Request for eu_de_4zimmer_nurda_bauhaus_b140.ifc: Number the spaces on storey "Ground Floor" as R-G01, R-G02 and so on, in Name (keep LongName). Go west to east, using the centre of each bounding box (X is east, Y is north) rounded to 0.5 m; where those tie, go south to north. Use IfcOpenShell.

First a look at what the model holds.

```python
import ifcopenshell
import ifcopenshell.util.element
import ifcopenshell.util.placement

model = ifcopenshell.open("eu_de_4zimmer_nurda_bauhaus_b140.ifc")
print(model.schema)
storey = next(s for s in model.by_type("IfcBuildingStorey") if s.Name == "Ground Floor")
spaces = [e for e in ifcopenshell.util.element.get_decomposition(storey) if e.is_a("IfcSpace")]
for e in sorted(spaces, key=lambda e: e.id()):
    origin = ifcopenshell.util.placement.get_local_placement(e.ObjectPlacement)[:3, 3]
    print(e.id(), e.Name, e.LongName, origin.round(2) + 0.0, sep=" | ")
```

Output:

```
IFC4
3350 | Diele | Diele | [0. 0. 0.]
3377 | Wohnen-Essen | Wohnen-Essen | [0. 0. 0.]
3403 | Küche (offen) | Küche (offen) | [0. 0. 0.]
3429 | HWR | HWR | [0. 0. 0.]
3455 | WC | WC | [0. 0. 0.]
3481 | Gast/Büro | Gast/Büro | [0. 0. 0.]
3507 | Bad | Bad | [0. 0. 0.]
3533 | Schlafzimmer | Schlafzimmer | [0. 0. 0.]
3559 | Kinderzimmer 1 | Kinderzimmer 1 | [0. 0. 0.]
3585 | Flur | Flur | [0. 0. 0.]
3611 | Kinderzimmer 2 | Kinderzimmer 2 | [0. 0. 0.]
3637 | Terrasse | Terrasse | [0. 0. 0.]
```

```python
import ifcopenshell
import ifcopenshell.geom
import ifcopenshell.util.element
import ifcopenshell.util.shape

model = ifcopenshell.open("eu_de_4zimmer_nurda_bauhaus_b140.ifc")
settings = ifcopenshell.geom.settings()
settings.set("use-world-coords", True)


def centre(element):
    shape = ifcopenshell.geom.create_shape(settings, element)
    return ifcopenshell.util.shape.get_bbox_centroid(shape.geometry)


storey = next(s for s in model.by_type("IfcBuildingStorey") if s.Name == "Ground Floor")
spaces = [e for e in ifcopenshell.util.element.get_decomposition(storey) if e.is_a("IfcSpace")]

# Insertion points can sit at a corner or the storey origin, so sort by the geometry (in metres).
centres = {e: centre(e) for e in spaces}
spaces.sort(key=lambda e: (round(centres[e][0] / 0.5), centres[e][1]))

for i, e in enumerate(spaces, start=1):
    number = f"R-G{i:02d}"
    e.Name = number
    print(e.id(), number)

model.write("eu_de_4zimmer_nurda_bauhaus_b140-out.ifc")
```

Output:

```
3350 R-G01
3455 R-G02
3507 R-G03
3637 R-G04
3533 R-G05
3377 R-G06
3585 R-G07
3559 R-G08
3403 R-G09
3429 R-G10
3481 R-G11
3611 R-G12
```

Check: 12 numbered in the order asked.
